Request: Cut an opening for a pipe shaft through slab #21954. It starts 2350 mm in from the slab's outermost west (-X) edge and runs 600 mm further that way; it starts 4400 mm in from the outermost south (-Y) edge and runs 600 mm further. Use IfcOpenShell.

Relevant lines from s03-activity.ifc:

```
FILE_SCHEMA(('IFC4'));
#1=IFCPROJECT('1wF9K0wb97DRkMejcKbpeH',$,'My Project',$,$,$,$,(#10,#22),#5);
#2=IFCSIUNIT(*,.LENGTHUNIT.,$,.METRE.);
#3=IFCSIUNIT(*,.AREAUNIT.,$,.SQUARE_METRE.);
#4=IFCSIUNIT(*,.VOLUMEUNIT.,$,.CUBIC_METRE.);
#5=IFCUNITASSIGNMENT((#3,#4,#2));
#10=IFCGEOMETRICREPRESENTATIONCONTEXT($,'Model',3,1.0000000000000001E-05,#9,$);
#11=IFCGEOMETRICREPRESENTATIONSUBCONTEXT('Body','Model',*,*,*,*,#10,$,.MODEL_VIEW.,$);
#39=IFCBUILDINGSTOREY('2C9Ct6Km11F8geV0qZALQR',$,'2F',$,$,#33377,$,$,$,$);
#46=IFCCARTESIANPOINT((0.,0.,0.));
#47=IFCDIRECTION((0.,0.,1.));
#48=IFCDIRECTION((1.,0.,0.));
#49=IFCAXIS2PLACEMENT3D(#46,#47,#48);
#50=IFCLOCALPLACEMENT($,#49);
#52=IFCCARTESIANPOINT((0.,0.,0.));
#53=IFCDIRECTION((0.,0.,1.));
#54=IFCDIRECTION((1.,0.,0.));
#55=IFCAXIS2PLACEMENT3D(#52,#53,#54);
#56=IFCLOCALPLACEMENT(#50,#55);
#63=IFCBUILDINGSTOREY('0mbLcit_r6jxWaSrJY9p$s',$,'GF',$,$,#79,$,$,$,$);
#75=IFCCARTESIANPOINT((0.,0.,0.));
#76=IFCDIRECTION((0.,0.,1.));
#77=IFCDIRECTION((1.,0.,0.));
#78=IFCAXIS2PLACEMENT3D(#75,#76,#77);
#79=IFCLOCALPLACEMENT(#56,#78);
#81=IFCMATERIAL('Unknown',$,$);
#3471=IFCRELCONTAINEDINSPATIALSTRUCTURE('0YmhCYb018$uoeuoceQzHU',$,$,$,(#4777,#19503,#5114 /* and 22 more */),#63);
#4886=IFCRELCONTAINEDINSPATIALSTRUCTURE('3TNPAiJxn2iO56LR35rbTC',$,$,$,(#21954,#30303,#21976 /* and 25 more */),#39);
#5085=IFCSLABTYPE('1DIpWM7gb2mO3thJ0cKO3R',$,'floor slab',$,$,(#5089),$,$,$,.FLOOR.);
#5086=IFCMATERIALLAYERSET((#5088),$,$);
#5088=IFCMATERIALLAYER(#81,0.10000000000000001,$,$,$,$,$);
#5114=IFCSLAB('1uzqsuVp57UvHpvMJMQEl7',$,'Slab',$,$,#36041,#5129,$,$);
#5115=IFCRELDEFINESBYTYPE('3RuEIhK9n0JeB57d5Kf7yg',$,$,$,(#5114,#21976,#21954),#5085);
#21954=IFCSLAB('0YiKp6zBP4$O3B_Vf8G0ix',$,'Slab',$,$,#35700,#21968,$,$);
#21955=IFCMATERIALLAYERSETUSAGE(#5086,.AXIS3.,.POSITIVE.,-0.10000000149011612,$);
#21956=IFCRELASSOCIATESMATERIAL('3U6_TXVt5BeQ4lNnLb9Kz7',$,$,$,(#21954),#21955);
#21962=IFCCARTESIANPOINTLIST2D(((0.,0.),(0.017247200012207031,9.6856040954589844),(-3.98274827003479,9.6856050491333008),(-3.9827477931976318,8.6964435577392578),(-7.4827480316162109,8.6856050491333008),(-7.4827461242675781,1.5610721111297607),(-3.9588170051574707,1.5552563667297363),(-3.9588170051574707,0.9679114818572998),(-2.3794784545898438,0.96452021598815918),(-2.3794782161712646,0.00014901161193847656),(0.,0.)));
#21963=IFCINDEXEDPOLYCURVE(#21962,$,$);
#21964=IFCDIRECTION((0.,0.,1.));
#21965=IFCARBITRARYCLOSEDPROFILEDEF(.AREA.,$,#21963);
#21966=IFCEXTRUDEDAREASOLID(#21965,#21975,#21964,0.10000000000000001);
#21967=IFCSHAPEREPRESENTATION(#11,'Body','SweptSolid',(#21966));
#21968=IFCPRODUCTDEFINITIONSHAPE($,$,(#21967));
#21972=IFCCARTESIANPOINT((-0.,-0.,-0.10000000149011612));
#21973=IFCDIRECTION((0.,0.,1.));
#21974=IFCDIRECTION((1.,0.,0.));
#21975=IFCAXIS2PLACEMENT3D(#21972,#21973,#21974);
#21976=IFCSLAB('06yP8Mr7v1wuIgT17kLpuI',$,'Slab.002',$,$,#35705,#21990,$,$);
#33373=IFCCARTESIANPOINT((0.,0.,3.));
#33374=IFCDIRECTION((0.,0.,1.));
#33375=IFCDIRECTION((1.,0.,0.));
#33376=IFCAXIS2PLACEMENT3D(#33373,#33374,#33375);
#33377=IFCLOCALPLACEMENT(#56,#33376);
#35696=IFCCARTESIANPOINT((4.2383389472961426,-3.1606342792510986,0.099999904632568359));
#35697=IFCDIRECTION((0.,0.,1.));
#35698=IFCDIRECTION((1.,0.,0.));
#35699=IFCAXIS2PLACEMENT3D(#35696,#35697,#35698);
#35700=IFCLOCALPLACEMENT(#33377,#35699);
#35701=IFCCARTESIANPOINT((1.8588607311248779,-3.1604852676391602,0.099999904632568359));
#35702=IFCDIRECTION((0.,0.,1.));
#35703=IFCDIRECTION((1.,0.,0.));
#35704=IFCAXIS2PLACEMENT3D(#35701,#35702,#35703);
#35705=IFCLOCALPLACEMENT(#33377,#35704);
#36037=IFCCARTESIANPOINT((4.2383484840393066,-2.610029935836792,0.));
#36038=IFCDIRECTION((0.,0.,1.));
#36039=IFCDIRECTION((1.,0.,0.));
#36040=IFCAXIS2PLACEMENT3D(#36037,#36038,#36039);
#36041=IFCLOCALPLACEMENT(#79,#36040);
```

```python
import numpy as np
import ifcopenshell
import ifcopenshell.api.feature
import ifcopenshell.api.geometry
import ifcopenshell.api.root
import ifcopenshell.geom
import ifcopenshell.util.placement
import ifcopenshell.util.representation
import ifcopenshell.util.shape
import ifcopenshell.util.unit

model = ifcopenshell.open("s03-activity.ifc")
unit_scale = ifcopenshell.util.unit.calculate_unit_scale(model)
settings = ifcopenshell.geom.settings()


def volume(element):
    """Net volume in cubic metres, openings subtracted."""
    shape = ifcopenshell.geom.create_shape(settings, element)
    return ifcopenshell.util.shape.get_volume(shape.geometry)


slab = model.by_guid("0YiKp6zBP4$O3B_Vf8G0ix")
before = volume(slab)

# Extent in the slab's own axes, in metres. The edges named are its -X and -Y sides.
slab_shape = ifcopenshell.geom.create_shape(settings, slab)
vertices = ifcopenshell.util.shape.get_vertices(slab_shape.geometry)
x_min, y_min, bottom = vertices.min(axis=0)
top = vertices[:, 2].max()

opening = ifcopenshell.api.root.create_entity(model, ifc_class="IfcOpeningElement", name="Pipe shaft opening", predefined_type="OPENING")
context = ifcopenshell.util.representation.get_context(model, "Model", "Body", "MODEL_VIEW")
width, depth = 0.6, 0.6
outline = [(0.0, 0.0), (width, 0.0), (width, depth), (0.0, depth), (0.0, 0.0)]
# Overshoot both faces by 50 mm so the cut is clean.
shape = ifcopenshell.api.geometry.add_slab_representation(
    model, context=context, depth=top - bottom + 0.1, polyline=outline
)
ifcopenshell.api.geometry.assign_representation(model, product=opening, representation=shape)

matrix = ifcopenshell.util.placement.get_local_placement(slab.ObjectPlacement)
matrix[:, 3] = matrix @ np.append(np.array([x_min + 2.35, y_min + 4.4, bottom - 0.05]) / unit_scale, 1.0)
ifcopenshell.api.geometry.edit_object_placement(model, product=opening, matrix=matrix, is_si=False)
ifcopenshell.api.feature.add_feature(model, feature=opening, element=slab)

after = volume(slab)

print(f"slab volume {before:.3f} -> {after:.3f} m3")

model.write("s03-activity-out.ifc")
```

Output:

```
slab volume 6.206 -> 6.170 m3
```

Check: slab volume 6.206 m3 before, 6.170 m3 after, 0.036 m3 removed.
